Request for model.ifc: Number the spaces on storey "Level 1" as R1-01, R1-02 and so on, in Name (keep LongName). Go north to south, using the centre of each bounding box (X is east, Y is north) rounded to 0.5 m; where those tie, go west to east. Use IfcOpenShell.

First a look at what the model holds.

```python
import ifcopenshell
import ifcopenshell.util.element
import ifcopenshell.util.placement

model = ifcopenshell.open("model.ifc")
print(model.schema)
storey = next(s for s in model.by_type("IfcBuildingStorey") if s.Name == "Level 1")
spaces = [e for e in ifcopenshell.util.element.get_decomposition(storey) if e.is_a("IfcSpace")]
for e in sorted(spaces, key=lambda e: e.id()):
    origin = ifcopenshell.util.placement.get_local_placement(e.ObjectPlacement)[:3, 3]
    print(e.id(), e.Name, e.LongName, origin.round(2) + 0.0, sep=" | ")
```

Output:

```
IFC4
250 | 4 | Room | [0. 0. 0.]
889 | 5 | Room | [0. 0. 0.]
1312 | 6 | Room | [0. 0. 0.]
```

```python
import ifcopenshell
import ifcopenshell.geom
import ifcopenshell.util.element
import ifcopenshell.util.shape

model = ifcopenshell.open("model.ifc")
settings = ifcopenshell.geom.settings()
settings.set("use-world-coords", True)


def centre(element):
    shape = ifcopenshell.geom.create_shape(settings, element)
    return ifcopenshell.util.shape.get_bbox_centroid(shape.geometry)


storey = next(s for s in model.by_type("IfcBuildingStorey") if s.Name == "Level 1")
spaces = [e for e in ifcopenshell.util.element.get_decomposition(storey) if e.is_a("IfcSpace")]

# Insertion points can sit at a corner or the storey origin, so sort by the geometry (in metres).
centres = {e: centre(e) for e in spaces}
spaces.sort(key=lambda e: (-round(centres[e][1] / 0.5), centres[e][0]))

for i, e in enumerate(spaces, start=1):
    number = f"R1-{i:02d}"
    e.Name = number
    print(e.id(), number)

model.write("model_edited.ifc")
```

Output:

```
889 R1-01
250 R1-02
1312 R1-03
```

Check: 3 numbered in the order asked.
